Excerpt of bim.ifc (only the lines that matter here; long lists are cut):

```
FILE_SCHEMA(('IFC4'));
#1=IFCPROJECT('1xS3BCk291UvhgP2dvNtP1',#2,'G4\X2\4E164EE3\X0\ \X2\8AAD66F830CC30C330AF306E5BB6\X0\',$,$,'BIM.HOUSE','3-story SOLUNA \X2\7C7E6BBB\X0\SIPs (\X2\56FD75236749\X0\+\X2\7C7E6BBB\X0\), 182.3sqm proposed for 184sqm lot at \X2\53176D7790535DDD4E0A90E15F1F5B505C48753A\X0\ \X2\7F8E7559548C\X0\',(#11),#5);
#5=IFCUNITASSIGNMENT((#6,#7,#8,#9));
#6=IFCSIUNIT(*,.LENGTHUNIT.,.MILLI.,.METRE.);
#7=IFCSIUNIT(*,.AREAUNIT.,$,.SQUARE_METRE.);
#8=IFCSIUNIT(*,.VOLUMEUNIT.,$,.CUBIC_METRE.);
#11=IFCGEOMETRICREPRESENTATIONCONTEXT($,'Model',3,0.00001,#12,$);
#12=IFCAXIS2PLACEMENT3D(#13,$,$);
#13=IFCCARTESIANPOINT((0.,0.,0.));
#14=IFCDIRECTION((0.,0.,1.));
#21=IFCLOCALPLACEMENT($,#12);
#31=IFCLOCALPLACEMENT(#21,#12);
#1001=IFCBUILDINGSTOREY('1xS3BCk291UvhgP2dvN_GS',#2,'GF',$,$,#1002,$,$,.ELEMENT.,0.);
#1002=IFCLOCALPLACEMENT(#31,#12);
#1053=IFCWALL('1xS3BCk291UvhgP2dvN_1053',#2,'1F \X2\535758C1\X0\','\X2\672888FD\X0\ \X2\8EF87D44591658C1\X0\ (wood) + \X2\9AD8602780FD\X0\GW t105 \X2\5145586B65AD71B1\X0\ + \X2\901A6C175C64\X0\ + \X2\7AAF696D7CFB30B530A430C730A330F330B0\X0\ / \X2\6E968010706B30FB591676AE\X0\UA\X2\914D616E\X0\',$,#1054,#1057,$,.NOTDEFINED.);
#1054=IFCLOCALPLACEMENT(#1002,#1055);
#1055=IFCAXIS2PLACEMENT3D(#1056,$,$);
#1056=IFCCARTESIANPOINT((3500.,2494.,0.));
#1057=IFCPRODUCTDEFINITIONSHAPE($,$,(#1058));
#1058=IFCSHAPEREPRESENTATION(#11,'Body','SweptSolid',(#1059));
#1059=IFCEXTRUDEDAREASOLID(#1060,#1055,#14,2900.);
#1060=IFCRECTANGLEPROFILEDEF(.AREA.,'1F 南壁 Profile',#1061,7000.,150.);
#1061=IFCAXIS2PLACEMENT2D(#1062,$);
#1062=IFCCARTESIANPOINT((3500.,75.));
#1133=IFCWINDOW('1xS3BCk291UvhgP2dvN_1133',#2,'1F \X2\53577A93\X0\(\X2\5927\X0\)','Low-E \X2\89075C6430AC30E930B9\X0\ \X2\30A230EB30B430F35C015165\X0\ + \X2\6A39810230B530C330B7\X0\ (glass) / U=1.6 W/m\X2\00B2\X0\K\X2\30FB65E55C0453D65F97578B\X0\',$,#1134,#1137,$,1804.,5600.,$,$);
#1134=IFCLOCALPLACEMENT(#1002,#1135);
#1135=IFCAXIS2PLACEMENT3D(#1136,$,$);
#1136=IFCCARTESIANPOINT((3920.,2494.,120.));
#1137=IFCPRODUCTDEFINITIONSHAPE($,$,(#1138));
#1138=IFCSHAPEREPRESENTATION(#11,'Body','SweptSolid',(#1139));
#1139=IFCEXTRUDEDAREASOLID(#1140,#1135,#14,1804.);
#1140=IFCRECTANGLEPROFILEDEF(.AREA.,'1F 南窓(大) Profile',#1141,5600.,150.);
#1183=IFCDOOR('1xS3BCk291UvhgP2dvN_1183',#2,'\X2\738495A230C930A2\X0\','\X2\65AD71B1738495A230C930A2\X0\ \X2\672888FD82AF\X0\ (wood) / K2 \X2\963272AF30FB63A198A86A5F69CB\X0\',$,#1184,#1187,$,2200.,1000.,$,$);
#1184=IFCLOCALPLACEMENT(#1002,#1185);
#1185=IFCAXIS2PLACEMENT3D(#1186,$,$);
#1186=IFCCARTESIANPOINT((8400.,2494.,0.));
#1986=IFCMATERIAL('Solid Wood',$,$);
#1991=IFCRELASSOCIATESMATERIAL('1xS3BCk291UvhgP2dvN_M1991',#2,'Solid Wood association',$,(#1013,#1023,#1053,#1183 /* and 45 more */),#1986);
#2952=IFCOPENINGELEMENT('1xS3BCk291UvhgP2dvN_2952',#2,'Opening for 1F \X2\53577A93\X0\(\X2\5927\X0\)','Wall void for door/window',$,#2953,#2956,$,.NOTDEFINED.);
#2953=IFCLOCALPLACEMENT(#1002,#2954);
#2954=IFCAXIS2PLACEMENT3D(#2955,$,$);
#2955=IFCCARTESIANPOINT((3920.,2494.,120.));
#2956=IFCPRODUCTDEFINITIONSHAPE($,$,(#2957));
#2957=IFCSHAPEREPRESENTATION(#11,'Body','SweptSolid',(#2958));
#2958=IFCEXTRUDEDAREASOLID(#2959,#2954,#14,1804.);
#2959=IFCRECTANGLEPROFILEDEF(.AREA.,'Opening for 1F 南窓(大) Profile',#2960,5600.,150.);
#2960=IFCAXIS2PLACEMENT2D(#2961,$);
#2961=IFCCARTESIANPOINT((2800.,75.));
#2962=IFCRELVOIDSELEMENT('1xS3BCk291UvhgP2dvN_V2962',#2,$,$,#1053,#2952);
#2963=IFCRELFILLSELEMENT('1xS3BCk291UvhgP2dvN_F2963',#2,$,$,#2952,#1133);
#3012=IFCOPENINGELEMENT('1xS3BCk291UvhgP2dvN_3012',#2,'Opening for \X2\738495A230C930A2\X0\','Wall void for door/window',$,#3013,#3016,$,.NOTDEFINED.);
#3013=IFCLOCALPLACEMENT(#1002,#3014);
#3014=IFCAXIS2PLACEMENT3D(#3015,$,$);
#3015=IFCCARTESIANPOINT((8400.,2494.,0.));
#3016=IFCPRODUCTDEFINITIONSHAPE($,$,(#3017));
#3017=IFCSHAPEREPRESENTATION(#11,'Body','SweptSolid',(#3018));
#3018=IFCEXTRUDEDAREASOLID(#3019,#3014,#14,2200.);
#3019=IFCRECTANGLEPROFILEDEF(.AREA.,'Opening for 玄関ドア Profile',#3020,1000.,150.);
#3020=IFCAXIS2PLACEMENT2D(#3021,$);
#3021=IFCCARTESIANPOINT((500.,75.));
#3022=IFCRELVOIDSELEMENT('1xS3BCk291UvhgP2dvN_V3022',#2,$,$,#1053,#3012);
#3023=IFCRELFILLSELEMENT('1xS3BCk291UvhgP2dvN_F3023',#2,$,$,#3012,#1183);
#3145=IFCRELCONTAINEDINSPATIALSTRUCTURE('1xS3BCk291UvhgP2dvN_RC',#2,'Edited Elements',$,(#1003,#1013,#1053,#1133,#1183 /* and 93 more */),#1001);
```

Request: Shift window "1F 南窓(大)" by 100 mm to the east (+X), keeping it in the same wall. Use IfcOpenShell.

```python
import ifcopenshell
import ifcopenshell.api.geometry
import ifcopenshell.util.placement

model = ifcopenshell.open("bim.ifc")

window = model.by_id(1133)
opening = window.FillsVoids[0].RelatingOpeningElement
wall = opening.VoidsElements[0].RelatingBuildingElement

wall_matrix = ifcopenshell.util.placement.get_local_placement(wall.ObjectPlacement)
shift = wall_matrix[:3, 0] * 100.0
before = ifcopenshell.util.placement.get_local_placement(window.ObjectPlacement)[:3, 3].copy()

# The window is not placed relative to its opening, so move both.
for product in (opening, window):
    matrix = ifcopenshell.util.placement.get_local_placement(product.ObjectPlacement)
    matrix[:3, 3] += shift
    ifcopenshell.api.geometry.edit_object_placement(model, product=product, matrix=matrix, is_si=False)

after = ifcopenshell.util.placement.get_local_placement(window.ObjectPlacement)[:3, 3]
print("window moved by", (after - before).round(3) + 0.0)

model.write("bim_edited.ifc")
```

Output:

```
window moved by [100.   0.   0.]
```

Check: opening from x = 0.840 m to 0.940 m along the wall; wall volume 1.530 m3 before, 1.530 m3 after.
